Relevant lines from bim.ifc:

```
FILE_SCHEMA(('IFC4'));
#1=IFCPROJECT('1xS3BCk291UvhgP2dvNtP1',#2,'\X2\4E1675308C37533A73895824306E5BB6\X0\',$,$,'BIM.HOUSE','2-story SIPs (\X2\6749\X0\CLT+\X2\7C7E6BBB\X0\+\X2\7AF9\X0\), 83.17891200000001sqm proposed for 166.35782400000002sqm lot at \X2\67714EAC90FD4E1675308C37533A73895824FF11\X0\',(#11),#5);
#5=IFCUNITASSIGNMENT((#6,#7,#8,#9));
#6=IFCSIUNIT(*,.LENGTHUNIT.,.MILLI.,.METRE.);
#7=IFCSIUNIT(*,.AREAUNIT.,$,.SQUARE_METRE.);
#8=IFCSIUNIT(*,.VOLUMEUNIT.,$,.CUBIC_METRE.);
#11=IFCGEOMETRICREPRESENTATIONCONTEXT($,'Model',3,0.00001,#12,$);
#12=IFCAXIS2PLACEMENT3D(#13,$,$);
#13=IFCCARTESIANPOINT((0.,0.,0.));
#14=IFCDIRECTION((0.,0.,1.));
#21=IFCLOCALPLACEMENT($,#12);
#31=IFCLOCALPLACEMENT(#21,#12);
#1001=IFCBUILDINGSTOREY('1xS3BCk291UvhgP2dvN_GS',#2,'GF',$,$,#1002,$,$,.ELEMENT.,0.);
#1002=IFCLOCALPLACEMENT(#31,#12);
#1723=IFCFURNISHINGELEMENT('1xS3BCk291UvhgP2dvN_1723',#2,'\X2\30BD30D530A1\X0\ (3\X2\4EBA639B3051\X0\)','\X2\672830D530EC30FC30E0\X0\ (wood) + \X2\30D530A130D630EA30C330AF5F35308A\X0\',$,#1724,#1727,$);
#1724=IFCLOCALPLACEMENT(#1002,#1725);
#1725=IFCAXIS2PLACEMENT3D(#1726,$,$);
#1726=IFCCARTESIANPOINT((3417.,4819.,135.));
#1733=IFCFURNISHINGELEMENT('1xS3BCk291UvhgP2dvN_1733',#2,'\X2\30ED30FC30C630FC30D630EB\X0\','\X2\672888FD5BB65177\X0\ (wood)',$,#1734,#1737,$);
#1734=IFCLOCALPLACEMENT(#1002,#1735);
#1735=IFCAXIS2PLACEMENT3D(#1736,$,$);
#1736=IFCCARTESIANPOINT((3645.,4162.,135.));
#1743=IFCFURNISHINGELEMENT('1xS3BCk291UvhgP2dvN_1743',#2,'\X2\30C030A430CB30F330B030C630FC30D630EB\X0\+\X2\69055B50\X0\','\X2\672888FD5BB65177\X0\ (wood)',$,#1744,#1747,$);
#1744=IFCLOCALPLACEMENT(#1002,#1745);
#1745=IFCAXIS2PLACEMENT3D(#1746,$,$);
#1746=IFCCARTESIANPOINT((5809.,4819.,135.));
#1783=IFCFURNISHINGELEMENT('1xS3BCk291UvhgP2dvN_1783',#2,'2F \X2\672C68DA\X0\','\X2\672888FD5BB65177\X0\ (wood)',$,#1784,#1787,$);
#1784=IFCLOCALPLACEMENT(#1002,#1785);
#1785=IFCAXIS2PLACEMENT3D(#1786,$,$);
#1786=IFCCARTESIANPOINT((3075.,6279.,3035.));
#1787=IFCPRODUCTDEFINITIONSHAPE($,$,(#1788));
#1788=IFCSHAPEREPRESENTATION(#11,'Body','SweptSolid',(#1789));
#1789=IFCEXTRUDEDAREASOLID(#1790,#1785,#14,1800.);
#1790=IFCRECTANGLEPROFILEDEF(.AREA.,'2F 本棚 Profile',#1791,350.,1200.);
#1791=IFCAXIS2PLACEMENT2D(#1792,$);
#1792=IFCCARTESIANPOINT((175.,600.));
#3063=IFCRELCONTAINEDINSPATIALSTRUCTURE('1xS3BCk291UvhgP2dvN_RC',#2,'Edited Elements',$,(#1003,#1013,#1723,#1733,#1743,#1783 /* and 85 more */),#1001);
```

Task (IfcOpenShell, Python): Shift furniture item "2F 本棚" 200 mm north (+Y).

```python
import ifcopenshell
import ifcopenshell.api.geometry
import ifcopenshell.util.placement
import ifcopenshell.util.unit

model = ifcopenshell.open("bim.ifc")
unit_scale = ifcopenshell.util.unit.calculate_unit_scale(model)

item = model.by_guid("1xS3BCk291UvhgP2dvN_1783")
matrix = ifcopenshell.util.placement.get_local_placement(item.ObjectPlacement)
matrix[1, 3] += 0.2 / unit_scale
ifcopenshell.api.geometry.edit_object_placement(model, product=item, matrix=matrix, is_si=False)

print(ifcopenshell.util.placement.get_local_placement(item.ObjectPlacement).round(3) + 0.0)

model.write("bim-out.ifc")
```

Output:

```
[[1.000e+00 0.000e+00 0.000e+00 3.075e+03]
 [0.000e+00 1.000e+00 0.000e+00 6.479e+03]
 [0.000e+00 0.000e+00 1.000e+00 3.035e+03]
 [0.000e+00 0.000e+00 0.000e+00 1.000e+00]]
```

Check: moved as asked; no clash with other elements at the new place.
